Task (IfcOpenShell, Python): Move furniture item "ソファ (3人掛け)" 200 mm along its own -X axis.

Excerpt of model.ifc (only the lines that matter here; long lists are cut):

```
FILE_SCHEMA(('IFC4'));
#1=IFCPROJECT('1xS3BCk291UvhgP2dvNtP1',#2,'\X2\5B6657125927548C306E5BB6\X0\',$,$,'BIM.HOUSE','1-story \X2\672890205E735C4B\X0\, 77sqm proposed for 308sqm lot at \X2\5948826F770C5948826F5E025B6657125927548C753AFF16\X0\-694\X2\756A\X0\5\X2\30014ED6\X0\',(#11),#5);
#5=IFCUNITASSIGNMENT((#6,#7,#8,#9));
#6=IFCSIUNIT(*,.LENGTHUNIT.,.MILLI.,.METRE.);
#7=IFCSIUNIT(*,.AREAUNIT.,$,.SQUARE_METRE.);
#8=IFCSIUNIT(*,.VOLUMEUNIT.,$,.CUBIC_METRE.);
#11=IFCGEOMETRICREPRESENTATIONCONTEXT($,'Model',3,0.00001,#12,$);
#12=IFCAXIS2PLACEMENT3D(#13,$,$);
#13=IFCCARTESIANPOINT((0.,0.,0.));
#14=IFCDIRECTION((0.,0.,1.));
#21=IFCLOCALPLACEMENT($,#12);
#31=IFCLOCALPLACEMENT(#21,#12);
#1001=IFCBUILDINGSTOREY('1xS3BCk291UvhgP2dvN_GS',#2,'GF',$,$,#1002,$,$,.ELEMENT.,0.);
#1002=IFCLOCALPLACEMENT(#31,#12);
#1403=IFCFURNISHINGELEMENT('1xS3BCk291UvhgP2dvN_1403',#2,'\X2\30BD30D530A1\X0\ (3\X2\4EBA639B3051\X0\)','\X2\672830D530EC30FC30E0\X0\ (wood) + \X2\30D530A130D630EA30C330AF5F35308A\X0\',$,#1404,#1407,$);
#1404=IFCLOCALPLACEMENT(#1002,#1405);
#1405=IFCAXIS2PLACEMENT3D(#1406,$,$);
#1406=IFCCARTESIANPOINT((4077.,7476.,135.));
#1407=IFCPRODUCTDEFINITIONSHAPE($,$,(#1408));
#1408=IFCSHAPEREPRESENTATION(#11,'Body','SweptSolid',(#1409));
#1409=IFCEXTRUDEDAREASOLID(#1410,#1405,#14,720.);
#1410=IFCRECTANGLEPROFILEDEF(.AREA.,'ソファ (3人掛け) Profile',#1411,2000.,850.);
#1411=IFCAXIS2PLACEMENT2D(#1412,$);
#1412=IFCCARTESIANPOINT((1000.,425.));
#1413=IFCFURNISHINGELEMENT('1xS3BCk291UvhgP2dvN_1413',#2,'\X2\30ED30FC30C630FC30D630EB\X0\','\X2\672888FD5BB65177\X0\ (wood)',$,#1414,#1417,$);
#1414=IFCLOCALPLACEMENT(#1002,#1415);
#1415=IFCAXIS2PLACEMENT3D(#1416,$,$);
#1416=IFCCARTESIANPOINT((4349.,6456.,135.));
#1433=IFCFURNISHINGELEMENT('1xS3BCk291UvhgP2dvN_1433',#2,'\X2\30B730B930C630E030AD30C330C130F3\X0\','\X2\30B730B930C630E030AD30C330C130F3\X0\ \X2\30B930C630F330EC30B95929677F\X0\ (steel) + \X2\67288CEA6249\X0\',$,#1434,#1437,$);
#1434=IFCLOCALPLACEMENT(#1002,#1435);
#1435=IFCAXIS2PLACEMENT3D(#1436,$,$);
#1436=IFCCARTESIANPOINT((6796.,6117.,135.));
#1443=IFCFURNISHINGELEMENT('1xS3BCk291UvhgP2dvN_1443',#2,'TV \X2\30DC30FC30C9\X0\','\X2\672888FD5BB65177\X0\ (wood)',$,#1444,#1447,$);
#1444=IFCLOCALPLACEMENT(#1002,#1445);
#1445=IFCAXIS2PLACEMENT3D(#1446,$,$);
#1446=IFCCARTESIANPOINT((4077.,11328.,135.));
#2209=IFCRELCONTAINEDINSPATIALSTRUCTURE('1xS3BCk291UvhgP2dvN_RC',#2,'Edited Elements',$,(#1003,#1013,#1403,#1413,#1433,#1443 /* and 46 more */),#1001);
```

```python
import ifcopenshell
import ifcopenshell.api.geometry
import ifcopenshell.util.placement

model = ifcopenshell.open("model.ifc")

item = model.by_id(1403)
matrix = ifcopenshell.util.placement.get_local_placement(item.ObjectPlacement)
matrix[:3, 3] -= matrix[:3, 0] * 200.0
ifcopenshell.api.geometry.edit_object_placement(model, product=item, matrix=matrix, is_si=False)

print(ifcopenshell.util.placement.get_local_placement(item.ObjectPlacement).round(3) + 0.0)

model.write("model-out.ifc")
```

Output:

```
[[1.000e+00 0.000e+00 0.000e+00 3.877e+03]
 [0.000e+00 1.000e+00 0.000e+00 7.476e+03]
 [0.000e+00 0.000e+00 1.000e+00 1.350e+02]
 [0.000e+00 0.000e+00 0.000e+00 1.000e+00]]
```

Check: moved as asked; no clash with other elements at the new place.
